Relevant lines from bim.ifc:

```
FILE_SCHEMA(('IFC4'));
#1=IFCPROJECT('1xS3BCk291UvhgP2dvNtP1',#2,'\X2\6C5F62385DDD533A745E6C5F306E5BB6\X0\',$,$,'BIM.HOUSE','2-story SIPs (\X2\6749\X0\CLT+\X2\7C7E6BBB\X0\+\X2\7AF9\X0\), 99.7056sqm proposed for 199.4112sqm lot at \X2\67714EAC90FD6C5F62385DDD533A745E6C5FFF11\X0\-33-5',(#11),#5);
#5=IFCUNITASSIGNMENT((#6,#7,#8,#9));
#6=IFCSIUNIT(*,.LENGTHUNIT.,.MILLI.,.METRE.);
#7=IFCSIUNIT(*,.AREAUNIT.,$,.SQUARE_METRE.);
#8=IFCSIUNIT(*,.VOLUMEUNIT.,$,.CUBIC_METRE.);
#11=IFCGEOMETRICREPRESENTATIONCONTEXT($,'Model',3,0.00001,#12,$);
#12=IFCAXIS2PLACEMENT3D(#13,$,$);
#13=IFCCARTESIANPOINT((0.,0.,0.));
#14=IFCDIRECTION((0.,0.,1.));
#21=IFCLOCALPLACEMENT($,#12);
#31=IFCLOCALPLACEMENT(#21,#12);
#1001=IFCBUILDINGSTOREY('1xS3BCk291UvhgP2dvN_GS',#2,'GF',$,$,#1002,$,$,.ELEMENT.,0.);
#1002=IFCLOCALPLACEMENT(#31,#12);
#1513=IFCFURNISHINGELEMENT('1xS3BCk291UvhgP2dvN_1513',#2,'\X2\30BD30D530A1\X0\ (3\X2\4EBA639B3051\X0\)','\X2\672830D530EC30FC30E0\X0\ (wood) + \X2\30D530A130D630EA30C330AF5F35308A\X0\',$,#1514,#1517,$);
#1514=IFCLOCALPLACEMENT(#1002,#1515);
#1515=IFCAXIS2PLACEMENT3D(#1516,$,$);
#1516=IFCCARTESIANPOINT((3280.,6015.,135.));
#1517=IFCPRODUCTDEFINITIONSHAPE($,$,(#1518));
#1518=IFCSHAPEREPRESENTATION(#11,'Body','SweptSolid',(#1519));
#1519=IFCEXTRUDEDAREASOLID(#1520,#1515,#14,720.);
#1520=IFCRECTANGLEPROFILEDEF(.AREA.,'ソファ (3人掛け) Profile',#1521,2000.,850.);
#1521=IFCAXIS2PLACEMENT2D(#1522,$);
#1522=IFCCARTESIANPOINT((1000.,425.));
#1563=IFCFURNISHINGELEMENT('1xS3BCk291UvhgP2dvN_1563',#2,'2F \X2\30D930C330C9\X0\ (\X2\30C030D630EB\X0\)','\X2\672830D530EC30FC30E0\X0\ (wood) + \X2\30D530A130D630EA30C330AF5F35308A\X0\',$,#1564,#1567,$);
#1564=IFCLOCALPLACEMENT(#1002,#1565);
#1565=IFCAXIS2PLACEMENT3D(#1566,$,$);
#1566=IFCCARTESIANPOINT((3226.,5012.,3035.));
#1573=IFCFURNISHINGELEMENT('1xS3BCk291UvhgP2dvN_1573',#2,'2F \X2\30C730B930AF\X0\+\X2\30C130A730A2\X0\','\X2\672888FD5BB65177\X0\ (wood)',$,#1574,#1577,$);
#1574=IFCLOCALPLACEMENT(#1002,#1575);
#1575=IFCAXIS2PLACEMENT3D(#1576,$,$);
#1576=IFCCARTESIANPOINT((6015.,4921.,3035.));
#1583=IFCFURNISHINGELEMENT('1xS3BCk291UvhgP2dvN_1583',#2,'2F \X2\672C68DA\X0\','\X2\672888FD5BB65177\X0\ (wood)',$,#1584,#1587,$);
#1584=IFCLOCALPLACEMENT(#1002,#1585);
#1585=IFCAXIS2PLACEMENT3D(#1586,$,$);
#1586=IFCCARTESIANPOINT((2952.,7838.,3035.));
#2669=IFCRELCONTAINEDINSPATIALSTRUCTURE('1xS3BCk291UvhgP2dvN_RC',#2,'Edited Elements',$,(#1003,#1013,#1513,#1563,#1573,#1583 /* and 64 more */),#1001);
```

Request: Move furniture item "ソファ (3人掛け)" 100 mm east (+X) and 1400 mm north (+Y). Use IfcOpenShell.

```python
import ifcopenshell
import ifcopenshell.api.geometry
import ifcopenshell.util.placement

model = ifcopenshell.open("bim.ifc")

item = model.by_guid("1xS3BCk291UvhgP2dvN_1513")
matrix = ifcopenshell.util.placement.get_local_placement(item.ObjectPlacement)
matrix[0, 3] += 100.0
matrix[1, 3] += 1400.0
ifcopenshell.api.geometry.edit_object_placement(model, product=item, matrix=matrix, is_si=False)

print(ifcopenshell.util.placement.get_local_placement(item.ObjectPlacement).round(3) + 0.0)

model.write("bim_updated.ifc")
```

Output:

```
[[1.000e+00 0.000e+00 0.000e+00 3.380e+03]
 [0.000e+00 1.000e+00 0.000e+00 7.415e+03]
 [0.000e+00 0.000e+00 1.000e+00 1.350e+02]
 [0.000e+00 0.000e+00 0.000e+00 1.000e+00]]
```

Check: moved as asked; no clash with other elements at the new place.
